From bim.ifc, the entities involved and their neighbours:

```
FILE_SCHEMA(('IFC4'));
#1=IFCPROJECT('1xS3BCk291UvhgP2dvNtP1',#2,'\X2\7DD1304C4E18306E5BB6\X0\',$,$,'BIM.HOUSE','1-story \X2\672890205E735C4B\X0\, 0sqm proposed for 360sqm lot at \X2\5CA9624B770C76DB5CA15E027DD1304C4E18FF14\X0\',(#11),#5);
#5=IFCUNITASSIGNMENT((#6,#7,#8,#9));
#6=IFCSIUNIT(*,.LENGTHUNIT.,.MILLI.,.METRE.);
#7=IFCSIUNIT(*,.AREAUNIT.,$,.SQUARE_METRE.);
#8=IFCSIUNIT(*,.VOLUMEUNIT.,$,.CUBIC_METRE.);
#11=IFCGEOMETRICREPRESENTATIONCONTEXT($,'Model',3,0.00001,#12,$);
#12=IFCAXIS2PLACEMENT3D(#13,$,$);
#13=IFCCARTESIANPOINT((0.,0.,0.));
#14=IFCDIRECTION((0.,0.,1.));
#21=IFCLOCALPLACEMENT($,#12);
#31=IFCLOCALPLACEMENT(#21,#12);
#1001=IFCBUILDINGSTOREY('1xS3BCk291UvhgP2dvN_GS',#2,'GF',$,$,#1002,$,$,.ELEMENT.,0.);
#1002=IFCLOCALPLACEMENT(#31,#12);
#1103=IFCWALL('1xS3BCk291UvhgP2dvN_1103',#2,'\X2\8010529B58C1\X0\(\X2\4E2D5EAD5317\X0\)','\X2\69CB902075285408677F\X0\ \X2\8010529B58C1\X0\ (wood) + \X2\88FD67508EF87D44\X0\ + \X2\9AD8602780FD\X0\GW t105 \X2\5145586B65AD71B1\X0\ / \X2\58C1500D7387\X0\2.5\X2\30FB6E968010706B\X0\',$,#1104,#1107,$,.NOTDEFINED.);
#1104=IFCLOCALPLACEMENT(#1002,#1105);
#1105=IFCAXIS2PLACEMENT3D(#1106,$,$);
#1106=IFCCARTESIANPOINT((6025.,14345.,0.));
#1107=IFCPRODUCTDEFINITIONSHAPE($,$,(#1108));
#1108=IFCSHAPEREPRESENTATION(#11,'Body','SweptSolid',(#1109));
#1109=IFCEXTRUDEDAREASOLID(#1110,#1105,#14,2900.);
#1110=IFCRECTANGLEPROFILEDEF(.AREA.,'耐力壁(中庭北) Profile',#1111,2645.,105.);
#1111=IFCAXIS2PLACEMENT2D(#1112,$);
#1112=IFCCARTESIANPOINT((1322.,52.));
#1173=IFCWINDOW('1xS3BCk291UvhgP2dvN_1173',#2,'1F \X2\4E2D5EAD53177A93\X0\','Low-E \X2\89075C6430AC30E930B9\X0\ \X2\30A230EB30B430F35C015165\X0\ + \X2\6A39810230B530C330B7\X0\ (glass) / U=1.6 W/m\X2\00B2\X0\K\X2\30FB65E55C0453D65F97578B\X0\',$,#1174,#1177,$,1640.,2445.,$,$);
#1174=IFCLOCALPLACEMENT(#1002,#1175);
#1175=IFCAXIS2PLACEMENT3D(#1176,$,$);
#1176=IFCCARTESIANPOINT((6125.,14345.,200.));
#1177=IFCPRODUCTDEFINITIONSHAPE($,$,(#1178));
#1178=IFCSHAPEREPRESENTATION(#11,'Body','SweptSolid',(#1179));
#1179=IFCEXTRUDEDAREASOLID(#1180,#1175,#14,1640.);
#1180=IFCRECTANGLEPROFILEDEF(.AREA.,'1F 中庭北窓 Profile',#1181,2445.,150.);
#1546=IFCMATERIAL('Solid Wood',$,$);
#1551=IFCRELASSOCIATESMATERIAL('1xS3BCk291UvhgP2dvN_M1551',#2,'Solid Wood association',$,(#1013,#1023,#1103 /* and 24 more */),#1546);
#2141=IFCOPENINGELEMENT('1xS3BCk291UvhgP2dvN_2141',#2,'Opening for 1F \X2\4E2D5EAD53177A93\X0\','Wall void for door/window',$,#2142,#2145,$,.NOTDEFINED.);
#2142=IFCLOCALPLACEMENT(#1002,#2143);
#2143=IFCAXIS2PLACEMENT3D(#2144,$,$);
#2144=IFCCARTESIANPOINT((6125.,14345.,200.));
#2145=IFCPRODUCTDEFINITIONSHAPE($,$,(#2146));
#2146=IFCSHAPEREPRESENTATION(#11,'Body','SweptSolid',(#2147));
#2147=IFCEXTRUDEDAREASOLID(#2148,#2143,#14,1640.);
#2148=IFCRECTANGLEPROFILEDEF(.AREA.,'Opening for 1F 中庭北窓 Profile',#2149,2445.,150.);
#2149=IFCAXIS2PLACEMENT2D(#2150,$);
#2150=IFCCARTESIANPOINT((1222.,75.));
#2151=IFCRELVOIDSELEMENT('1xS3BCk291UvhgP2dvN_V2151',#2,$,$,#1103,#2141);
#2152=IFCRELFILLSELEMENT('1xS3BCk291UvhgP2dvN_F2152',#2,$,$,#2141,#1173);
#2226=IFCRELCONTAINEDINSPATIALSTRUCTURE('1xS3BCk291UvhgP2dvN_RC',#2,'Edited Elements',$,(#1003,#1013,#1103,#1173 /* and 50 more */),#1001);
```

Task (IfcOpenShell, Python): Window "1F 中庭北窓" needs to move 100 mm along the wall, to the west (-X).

```python
import ifcopenshell
import ifcopenshell.api.geometry
import ifcopenshell.util.placement
import ifcopenshell.util.unit

model = ifcopenshell.open("bim.ifc")
unit_scale = ifcopenshell.util.unit.calculate_unit_scale(model)

window = model.by_id(1173)
opening = window.FillsVoids[0].RelatingOpeningElement
wall = opening.VoidsElements[0].RelatingBuildingElement

wall_matrix = ifcopenshell.util.placement.get_local_placement(wall.ObjectPlacement)
shift = wall_matrix[:3, 0] * -0.1 / unit_scale
before = ifcopenshell.util.placement.get_local_placement(window.ObjectPlacement)[:3, 3].copy()

# The window is not placed relative to its opening, so move both.
for product in (opening, window):
    matrix = ifcopenshell.util.placement.get_local_placement(product.ObjectPlacement)
    matrix[:3, 3] += shift
    ifcopenshell.api.geometry.edit_object_placement(model, product=product, matrix=matrix, is_si=False)

after = ifcopenshell.util.placement.get_local_placement(window.ObjectPlacement)[:3, 3]
print("window moved by", (after - before).round(3) + 0.0)

model.write("bim-out.ifc")
```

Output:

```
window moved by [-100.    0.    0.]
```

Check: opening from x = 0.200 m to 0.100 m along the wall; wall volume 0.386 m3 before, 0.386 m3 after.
